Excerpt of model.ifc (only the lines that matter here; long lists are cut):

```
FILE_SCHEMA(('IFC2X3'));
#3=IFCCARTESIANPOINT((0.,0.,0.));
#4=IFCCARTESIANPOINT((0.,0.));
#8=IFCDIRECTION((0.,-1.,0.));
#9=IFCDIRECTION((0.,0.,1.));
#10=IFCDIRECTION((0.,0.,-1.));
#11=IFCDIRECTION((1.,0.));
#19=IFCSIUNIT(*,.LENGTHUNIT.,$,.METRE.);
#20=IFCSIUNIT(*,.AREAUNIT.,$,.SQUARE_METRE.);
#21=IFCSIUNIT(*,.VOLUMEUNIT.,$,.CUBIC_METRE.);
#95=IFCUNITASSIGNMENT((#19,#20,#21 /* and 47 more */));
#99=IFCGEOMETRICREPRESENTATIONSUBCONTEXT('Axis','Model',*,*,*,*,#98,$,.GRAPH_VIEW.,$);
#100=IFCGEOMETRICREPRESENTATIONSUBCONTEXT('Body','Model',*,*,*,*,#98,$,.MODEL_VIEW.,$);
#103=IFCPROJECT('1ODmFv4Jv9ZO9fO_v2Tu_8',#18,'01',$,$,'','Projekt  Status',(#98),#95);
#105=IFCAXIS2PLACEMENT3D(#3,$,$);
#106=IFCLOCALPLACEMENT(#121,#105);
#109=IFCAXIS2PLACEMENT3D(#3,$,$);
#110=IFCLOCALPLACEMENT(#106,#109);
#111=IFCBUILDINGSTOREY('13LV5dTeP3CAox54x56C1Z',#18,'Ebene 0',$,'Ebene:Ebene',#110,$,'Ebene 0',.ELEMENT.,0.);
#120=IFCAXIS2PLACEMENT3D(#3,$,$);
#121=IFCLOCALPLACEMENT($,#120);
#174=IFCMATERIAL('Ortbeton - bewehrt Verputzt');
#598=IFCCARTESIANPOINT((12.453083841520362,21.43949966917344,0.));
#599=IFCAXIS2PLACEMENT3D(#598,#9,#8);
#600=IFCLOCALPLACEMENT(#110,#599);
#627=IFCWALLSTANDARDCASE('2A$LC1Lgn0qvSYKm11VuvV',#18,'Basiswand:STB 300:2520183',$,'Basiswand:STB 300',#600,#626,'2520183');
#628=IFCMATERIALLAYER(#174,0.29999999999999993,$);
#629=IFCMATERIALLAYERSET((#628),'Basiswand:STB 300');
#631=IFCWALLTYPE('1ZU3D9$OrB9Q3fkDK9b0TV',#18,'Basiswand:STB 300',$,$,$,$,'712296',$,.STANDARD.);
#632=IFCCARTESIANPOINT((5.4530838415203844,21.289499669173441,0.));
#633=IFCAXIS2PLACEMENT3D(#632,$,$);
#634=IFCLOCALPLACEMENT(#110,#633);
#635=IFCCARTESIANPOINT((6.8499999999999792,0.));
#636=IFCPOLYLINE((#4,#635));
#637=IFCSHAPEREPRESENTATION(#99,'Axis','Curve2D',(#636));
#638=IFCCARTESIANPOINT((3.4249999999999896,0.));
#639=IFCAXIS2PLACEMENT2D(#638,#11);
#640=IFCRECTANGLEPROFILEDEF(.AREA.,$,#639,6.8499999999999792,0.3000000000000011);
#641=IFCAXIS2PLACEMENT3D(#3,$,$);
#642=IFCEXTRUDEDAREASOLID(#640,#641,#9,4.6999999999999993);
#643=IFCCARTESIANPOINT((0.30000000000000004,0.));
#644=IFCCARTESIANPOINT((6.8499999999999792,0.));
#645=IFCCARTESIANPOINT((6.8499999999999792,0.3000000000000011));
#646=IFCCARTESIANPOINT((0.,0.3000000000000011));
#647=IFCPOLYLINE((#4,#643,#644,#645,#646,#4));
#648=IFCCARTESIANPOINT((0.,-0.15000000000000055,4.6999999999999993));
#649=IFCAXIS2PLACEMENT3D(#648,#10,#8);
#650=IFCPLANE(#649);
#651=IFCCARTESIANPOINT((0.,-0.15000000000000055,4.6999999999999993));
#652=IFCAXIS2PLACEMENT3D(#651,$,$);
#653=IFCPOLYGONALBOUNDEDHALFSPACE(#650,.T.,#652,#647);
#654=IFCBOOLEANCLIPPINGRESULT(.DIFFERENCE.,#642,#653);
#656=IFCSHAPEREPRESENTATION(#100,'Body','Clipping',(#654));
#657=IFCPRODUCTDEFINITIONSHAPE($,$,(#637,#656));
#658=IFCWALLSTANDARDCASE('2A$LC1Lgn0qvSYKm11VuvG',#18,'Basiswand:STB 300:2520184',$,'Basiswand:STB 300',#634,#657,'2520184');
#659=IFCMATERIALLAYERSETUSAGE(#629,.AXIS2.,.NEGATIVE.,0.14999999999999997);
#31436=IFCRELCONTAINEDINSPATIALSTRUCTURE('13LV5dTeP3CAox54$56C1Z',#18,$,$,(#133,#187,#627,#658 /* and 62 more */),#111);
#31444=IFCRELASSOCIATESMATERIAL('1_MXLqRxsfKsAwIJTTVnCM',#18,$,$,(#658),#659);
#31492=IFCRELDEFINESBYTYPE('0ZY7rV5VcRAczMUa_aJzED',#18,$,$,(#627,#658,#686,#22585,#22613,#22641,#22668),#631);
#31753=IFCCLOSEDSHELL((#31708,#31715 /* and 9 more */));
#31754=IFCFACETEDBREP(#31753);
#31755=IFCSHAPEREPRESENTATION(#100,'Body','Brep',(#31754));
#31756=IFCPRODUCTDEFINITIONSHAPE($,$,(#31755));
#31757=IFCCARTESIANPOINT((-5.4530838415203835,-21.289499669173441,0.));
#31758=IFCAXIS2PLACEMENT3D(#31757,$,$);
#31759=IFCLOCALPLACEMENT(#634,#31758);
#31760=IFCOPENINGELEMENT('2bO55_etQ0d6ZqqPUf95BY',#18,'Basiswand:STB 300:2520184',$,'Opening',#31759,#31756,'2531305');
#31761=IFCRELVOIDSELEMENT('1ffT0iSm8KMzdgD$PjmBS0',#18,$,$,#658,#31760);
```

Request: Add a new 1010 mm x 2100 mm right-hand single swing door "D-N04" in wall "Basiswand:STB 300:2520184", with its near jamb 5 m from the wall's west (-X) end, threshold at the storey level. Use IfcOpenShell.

```python
import numpy as np
import ifcopenshell
import ifcopenshell.api.feature
import ifcopenshell.api.geometry
import ifcopenshell.api.root
import ifcopenshell.api.spatial
import ifcopenshell.api.type
import ifcopenshell.geom
import ifcopenshell.util.element
import ifcopenshell.util.placement
import ifcopenshell.util.representation
import ifcopenshell.util.shape
import ifcopenshell.util.unit

model = ifcopenshell.open("model.ifc")
unit_scale = ifcopenshell.util.unit.calculate_unit_scale(model)
settings = ifcopenshell.geom.settings()


def volume(element):
    """Net volume in cubic metres, openings subtracted."""
    shape = ifcopenshell.geom.create_shape(settings, element)
    return ifcopenshell.util.shape.get_volume(shape.geometry)


wall = model.by_id(658)
storey = ifcopenshell.util.element.get_container(wall, ifc_class="IfcBuildingStorey")
context = ifcopenshell.util.representation.get_context(model, "Model", "Body", "MODEL_VIEW")
before = volume(wall)

width, height, from_end, sill = 1.01, 2.1, 5, 0.0  # metres

# The wall runs along its own X axis, and the end named is its -X end.
wall_shape = ifcopenshell.geom.create_shape(settings, wall)
x, y, z = ifcopenshell.util.shape.get_vertices(wall_shape.geometry).T
start = x.min() + from_end
face, thickness = float(y.min()), float(y.max() - y.min())
wall_matrix = ifcopenshell.util.placement.get_local_placement(wall.ObjectPlacement)
level = ifcopenshell.util.placement.get_local_placement(storey.ObjectPlacement)[2, 3]


def in_wall(x, y):
    """Placement at x, y metres in the wall's axes, at sill height."""
    matrix = wall_matrix.copy()
    matrix[:, 3] = wall_matrix @ np.array([x / unit_scale, y / unit_scale, 0.0, 1.0])
    matrix[2, 3] = level + sill / unit_scale
    return matrix


# Opening: a box that overshoots both wall faces by 50 mm.
opening = ifcopenshell.api.root.create_entity(model, ifc_class="IfcOpeningElement")
box = ifcopenshell.api.geometry.add_wall_representation(
    model, context=context, length=width, height=height, thickness=thickness + 0.1
)
ifcopenshell.api.geometry.assign_representation(model, product=opening, representation=box)
ifcopenshell.api.geometry.edit_object_placement(model, product=opening, matrix=in_wall(start, face - 0.05), is_si=False)
ifcopenshell.api.feature.add_feature(model, feature=opening, element=wall)

door = ifcopenshell.api.root.create_entity(model, ifc_class="IfcDoor", name="D-N04")
door.OverallWidth, door.OverallHeight = width / unit_scale, height / unit_scale
body = ifcopenshell.api.geometry.add_door_representation(
    model,
    context=context,
    overall_width=door.OverallWidth,
    overall_height=door.OverallHeight,
    operation_type="SINGLE_SWING_RIGHT",
    lining_properties={"LiningDepth": thickness / unit_scale, "ThresholdDepth": thickness / unit_scale},
)
ifcopenshell.api.geometry.assign_representation(model, product=door, representation=body)
ifcopenshell.api.spatial.assign_container(model, products=[door], relating_structure=storey)
fills = ifcopenshell.api.feature.add_filling(model, opening=opening, element=door)
fills.OwnerHistory = door.OwnerHistory  # required in IFC2X3

# IFC2X3 keeps the operation on the door style.
style = ifcopenshell.api.root.create_entity(model, ifc_class="IfcDoorStyle", name="D-N04")
style.OperationType, style.ConstructionType = "SINGLE_SWING_RIGHT", "NOTDEFINED"
style.ParameterTakesPrecedence = style.Sizeable = False
ifcopenshell.api.type.assign_type(model, related_objects=[door], relating_type=style)

# The lining spans the wall, so the door starts at the wall face.
ifcopenshell.api.geometry.edit_object_placement(model, product=door, matrix=in_wall(start, face), is_si=False)

after = volume(wall)

print(f"wall volume {before:.3f} -> {after:.3f} m3")

model.write("model-out.ifc")
```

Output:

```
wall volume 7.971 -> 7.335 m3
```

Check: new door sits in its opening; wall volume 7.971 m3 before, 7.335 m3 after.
